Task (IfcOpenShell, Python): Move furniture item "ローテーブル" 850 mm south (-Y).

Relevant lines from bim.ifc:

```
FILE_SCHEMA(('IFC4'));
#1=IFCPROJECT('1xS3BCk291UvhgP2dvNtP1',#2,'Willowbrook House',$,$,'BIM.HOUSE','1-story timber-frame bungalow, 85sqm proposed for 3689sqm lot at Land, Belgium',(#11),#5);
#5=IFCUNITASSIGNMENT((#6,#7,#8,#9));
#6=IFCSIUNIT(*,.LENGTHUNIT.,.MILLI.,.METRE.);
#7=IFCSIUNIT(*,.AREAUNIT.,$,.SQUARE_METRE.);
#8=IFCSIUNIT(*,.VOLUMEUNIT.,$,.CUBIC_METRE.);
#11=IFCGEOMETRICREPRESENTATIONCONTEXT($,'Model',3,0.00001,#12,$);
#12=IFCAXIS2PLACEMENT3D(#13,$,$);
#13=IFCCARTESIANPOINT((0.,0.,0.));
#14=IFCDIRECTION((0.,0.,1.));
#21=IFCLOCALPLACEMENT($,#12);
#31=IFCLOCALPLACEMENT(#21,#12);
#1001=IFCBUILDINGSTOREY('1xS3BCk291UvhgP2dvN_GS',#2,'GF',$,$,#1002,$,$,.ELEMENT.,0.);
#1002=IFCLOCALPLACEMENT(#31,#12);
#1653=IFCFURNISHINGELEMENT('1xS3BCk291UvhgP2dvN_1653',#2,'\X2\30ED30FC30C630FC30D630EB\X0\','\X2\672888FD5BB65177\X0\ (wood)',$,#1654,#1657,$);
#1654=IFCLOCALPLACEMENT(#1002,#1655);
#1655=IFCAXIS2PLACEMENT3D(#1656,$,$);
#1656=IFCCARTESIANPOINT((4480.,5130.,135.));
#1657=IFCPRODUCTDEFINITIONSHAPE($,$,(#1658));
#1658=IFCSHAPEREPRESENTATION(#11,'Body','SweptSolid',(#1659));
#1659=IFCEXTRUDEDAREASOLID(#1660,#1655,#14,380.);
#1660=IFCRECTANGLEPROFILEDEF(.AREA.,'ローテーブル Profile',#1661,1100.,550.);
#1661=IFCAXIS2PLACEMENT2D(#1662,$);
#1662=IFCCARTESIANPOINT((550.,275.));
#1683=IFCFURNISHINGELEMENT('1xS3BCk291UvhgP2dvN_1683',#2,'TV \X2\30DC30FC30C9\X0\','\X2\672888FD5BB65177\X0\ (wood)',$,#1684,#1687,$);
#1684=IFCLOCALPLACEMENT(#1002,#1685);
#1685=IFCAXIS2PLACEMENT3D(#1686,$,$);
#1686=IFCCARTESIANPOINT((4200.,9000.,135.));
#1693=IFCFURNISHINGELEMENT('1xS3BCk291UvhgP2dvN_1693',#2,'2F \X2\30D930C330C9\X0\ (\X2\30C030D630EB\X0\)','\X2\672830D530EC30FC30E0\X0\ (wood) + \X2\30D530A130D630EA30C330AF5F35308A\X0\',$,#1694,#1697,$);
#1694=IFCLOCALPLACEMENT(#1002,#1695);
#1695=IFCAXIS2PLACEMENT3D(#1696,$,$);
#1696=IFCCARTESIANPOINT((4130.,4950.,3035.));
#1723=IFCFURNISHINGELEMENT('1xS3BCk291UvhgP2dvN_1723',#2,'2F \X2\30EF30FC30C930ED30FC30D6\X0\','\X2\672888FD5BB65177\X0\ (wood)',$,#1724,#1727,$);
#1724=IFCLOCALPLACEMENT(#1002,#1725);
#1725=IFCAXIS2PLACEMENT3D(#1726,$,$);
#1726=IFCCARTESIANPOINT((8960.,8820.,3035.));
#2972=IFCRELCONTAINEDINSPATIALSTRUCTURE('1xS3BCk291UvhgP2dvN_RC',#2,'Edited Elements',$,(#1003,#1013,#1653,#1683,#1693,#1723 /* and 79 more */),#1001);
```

```python
import ifcopenshell
import ifcopenshell.api.geometry
import ifcopenshell.util.placement
import ifcopenshell.util.unit

model = ifcopenshell.open("bim.ifc")
unit_scale = ifcopenshell.util.unit.calculate_unit_scale(model)

item = model.by_id(1653)
matrix = ifcopenshell.util.placement.get_local_placement(item.ObjectPlacement)
matrix[1, 3] -= 0.85 / unit_scale
ifcopenshell.api.geometry.edit_object_placement(model, product=item, matrix=matrix, is_si=False)

print(ifcopenshell.util.placement.get_local_placement(item.ObjectPlacement).round(3) + 0.0)

model.write("bim_edited.ifc")
```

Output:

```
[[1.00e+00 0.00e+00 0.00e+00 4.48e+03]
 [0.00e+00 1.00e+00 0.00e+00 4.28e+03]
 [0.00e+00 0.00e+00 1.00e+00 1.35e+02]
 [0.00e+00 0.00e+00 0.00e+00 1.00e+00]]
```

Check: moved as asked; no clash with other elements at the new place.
